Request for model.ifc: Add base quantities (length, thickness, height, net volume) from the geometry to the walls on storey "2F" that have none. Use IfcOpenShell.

First a look at what the model holds.

```python
import ifcopenshell
import ifcopenshell.util.element
import ifcopenshell.util.unit

model = ifcopenshell.open("model.ifc")
print(model.schema)
for unit_type in ("LENGTHUNIT", "AREAUNIT", "VOLUMEUNIT"):
    print(unit_type, ifcopenshell.util.unit.calculate_unit_scale(model, unit_type))
storey = next(s for s in model.by_type("IfcBuildingStorey") if s.Name == "2F")
walls = [e for e in ifcopenshell.util.element.get_decomposition(storey) if e.is_a("IfcWall")]
for e in sorted(walls, key=lambda e: e.id()):
    print(e.id(), e.is_a(), e.Name, list(ifcopenshell.util.element.get_psets(e, qtos_only=True)), sep=" | ")
```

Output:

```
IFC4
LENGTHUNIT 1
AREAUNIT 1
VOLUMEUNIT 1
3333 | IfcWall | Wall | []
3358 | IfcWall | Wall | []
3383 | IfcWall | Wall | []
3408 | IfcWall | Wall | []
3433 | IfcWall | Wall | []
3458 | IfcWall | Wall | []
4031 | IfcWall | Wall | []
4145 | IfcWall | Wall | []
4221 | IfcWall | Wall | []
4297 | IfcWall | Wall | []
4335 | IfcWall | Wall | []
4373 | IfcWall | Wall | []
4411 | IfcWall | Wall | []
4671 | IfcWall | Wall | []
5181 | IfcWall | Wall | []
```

```python
import ifcopenshell
import ifcopenshell.api.pset
import ifcopenshell.geom
import ifcopenshell.util.element
import ifcopenshell.util.shape
import ifcopenshell.util.unit

model = ifcopenshell.open("model.ifc")
unit_scale = ifcopenshell.util.unit.calculate_unit_scale(model)
volume_scale = ifcopenshell.util.unit.calculate_unit_scale(model, "VOLUMEUNIT")
settings = ifcopenshell.geom.settings()

storey = next(s for s in model.by_type("IfcBuildingStorey") if s.Name == "2F")
walls = [e for e in ifcopenshell.util.element.get_decomposition(storey) if e.is_a("IfcWall")]

for e in sorted(walls, key=lambda e: e.id()):
    if ifcopenshell.util.element.get_psets(e, qtos_only=True, should_inherit=False):
        continue
    # Geometry comes back in metres, in the element's own axes.
    shape = ifcopenshell.geom.create_shape(settings, e)
    values = {
        "Length": ifcopenshell.util.shape.get_x(shape.geometry) / unit_scale,
        "Width": ifcopenshell.util.shape.get_y(shape.geometry) / unit_scale,
        "Height": ifcopenshell.util.shape.get_z(shape.geometry) / unit_scale,
        "NetVolume": ifcopenshell.util.shape.get_volume(shape.geometry) / volume_scale,
    }
    qto = ifcopenshell.api.pset.add_qto(model, product=e, name="Qto_WallBaseQuantities")
    ifcopenshell.api.pset.edit_qto(model, qto=qto, properties=values)
    print(e.id(), {k: round(v, 3) for k, v in values.items()})

model.write("model_v2.ifc")
```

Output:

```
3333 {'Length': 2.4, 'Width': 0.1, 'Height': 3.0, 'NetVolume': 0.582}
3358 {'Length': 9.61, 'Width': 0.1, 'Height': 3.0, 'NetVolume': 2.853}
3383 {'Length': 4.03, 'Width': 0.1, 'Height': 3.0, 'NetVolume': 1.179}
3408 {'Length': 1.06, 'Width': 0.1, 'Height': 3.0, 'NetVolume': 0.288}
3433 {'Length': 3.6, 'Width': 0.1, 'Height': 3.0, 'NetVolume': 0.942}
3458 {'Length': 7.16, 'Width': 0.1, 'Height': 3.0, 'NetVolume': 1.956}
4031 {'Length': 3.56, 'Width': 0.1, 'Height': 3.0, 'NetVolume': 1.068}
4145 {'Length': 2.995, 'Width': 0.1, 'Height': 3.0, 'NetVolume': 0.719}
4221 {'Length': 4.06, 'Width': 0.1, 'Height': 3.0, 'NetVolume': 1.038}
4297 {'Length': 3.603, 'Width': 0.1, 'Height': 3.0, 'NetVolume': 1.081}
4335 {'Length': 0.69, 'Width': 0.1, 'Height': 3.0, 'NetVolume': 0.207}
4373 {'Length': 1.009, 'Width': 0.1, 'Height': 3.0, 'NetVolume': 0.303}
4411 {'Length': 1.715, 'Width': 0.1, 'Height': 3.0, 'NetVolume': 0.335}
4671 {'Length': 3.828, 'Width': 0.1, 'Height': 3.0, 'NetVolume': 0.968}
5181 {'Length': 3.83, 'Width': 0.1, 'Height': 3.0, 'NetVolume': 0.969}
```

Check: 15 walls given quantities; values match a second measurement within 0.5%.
